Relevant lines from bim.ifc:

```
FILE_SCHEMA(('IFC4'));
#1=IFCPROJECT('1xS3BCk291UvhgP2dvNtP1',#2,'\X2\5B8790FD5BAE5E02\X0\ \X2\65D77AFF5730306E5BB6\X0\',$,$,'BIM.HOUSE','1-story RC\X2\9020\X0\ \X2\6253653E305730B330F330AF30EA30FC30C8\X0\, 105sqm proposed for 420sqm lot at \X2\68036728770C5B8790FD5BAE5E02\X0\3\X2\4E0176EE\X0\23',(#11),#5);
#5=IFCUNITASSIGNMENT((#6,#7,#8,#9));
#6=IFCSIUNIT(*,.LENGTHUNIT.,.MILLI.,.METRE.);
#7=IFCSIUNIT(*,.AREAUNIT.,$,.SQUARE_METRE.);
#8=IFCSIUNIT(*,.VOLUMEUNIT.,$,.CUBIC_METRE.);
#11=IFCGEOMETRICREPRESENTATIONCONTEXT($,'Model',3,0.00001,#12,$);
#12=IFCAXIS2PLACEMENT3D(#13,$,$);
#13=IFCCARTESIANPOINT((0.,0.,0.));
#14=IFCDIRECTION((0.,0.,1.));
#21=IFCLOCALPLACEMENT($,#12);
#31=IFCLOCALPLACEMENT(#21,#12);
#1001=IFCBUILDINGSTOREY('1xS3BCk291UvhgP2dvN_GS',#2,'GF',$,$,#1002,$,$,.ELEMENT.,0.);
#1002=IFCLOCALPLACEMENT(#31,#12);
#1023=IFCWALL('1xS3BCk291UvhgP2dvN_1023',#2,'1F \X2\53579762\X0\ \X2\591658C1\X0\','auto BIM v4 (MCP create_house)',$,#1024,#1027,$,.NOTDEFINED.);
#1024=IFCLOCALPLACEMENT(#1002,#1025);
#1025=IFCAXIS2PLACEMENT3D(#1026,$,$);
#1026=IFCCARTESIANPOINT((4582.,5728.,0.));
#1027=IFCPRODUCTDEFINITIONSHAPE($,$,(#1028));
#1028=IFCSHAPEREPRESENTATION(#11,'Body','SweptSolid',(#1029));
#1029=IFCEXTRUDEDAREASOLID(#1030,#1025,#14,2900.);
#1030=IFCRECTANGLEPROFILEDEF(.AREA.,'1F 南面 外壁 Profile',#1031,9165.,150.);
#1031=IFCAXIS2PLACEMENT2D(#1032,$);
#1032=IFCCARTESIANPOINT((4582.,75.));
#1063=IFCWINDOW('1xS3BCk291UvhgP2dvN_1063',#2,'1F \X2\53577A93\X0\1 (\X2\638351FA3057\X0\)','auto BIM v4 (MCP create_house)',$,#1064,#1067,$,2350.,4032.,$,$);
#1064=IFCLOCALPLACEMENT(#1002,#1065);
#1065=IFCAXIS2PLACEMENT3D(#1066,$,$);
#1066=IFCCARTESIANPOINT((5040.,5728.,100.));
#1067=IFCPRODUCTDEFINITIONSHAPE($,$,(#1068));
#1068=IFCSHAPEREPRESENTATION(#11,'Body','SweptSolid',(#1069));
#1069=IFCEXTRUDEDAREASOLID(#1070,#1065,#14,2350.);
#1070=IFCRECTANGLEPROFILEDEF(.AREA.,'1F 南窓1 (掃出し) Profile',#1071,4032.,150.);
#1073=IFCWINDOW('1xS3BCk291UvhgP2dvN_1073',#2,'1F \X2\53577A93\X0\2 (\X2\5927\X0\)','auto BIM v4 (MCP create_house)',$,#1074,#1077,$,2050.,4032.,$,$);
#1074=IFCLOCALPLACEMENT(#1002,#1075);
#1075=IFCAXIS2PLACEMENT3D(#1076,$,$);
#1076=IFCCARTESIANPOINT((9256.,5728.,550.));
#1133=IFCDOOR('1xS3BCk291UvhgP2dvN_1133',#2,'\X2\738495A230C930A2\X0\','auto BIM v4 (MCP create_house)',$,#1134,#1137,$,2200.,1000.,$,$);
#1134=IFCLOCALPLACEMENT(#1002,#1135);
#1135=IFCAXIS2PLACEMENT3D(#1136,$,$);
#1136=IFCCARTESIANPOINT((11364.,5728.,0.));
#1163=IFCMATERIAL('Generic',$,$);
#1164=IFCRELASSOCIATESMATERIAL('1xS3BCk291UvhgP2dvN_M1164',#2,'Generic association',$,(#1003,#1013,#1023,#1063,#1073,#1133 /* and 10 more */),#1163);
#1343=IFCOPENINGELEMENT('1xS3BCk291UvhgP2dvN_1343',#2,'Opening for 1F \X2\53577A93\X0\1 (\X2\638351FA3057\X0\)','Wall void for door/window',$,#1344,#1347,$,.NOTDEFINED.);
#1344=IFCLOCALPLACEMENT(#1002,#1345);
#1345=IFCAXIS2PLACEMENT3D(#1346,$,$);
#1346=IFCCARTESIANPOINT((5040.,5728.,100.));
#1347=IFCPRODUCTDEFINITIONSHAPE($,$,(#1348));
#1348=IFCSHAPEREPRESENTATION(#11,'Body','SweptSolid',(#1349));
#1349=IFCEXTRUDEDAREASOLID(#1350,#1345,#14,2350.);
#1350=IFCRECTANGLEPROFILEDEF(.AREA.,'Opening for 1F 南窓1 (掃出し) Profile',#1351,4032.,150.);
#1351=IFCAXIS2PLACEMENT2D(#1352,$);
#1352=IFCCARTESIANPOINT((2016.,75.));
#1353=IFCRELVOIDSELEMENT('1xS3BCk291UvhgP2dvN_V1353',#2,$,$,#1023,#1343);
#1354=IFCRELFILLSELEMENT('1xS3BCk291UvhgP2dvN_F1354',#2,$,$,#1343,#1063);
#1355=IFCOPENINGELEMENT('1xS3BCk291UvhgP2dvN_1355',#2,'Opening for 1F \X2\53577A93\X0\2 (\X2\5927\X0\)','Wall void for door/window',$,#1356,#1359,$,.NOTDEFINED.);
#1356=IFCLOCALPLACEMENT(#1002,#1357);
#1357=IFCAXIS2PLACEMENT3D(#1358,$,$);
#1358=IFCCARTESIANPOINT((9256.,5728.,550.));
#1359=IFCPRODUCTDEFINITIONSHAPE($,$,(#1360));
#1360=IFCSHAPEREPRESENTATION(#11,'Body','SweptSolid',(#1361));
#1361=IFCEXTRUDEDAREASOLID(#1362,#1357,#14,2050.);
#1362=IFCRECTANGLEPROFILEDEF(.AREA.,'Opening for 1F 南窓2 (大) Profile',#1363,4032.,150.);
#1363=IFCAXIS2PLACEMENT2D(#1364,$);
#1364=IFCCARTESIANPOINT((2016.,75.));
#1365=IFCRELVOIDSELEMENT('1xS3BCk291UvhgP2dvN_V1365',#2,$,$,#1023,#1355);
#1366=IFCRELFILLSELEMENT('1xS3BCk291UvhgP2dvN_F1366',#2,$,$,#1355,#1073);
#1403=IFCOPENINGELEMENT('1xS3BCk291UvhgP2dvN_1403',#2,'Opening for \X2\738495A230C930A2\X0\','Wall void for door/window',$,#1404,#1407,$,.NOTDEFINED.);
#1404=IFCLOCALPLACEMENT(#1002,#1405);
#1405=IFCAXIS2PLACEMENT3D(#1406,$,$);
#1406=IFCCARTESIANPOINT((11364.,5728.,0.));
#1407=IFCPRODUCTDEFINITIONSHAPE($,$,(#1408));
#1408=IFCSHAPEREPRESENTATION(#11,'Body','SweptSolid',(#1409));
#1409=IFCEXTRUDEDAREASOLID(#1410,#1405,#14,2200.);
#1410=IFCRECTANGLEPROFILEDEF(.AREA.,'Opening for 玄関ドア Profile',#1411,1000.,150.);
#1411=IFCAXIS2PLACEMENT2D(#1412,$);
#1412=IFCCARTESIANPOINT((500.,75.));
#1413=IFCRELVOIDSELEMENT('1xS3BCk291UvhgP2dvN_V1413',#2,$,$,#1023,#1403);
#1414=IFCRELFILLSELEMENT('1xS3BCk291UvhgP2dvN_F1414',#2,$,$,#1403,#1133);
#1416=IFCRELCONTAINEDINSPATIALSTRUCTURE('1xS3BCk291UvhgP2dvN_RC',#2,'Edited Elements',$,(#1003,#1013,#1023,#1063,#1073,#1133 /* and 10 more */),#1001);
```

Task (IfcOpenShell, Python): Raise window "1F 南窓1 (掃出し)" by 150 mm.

```python
import numpy as np
import ifcopenshell
import ifcopenshell.api.geometry
import ifcopenshell.util.placement
import ifcopenshell.util.unit

model = ifcopenshell.open("bim.ifc")
unit_scale = ifcopenshell.util.unit.calculate_unit_scale(model)

window = model.by_guid("1xS3BCk291UvhgP2dvN_1063")
opening = window.FillsVoids[0].RelatingOpeningElement
dz = 150.0

shift = np.array([0.0, 0.0, dz])
# The window is not placed relative to its opening, so move both.
for product in (opening, window):
    matrix = ifcopenshell.util.placement.get_local_placement(product.ObjectPlacement)
    matrix[:3, 3] += shift
    ifcopenshell.api.geometry.edit_object_placement(model, product=product, matrix=matrix, is_si=False)

print(f"moved by {dz * unit_scale:+.3f} m")

model.write("bim_v2.ifc")
```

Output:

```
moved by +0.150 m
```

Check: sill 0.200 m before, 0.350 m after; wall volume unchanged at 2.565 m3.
